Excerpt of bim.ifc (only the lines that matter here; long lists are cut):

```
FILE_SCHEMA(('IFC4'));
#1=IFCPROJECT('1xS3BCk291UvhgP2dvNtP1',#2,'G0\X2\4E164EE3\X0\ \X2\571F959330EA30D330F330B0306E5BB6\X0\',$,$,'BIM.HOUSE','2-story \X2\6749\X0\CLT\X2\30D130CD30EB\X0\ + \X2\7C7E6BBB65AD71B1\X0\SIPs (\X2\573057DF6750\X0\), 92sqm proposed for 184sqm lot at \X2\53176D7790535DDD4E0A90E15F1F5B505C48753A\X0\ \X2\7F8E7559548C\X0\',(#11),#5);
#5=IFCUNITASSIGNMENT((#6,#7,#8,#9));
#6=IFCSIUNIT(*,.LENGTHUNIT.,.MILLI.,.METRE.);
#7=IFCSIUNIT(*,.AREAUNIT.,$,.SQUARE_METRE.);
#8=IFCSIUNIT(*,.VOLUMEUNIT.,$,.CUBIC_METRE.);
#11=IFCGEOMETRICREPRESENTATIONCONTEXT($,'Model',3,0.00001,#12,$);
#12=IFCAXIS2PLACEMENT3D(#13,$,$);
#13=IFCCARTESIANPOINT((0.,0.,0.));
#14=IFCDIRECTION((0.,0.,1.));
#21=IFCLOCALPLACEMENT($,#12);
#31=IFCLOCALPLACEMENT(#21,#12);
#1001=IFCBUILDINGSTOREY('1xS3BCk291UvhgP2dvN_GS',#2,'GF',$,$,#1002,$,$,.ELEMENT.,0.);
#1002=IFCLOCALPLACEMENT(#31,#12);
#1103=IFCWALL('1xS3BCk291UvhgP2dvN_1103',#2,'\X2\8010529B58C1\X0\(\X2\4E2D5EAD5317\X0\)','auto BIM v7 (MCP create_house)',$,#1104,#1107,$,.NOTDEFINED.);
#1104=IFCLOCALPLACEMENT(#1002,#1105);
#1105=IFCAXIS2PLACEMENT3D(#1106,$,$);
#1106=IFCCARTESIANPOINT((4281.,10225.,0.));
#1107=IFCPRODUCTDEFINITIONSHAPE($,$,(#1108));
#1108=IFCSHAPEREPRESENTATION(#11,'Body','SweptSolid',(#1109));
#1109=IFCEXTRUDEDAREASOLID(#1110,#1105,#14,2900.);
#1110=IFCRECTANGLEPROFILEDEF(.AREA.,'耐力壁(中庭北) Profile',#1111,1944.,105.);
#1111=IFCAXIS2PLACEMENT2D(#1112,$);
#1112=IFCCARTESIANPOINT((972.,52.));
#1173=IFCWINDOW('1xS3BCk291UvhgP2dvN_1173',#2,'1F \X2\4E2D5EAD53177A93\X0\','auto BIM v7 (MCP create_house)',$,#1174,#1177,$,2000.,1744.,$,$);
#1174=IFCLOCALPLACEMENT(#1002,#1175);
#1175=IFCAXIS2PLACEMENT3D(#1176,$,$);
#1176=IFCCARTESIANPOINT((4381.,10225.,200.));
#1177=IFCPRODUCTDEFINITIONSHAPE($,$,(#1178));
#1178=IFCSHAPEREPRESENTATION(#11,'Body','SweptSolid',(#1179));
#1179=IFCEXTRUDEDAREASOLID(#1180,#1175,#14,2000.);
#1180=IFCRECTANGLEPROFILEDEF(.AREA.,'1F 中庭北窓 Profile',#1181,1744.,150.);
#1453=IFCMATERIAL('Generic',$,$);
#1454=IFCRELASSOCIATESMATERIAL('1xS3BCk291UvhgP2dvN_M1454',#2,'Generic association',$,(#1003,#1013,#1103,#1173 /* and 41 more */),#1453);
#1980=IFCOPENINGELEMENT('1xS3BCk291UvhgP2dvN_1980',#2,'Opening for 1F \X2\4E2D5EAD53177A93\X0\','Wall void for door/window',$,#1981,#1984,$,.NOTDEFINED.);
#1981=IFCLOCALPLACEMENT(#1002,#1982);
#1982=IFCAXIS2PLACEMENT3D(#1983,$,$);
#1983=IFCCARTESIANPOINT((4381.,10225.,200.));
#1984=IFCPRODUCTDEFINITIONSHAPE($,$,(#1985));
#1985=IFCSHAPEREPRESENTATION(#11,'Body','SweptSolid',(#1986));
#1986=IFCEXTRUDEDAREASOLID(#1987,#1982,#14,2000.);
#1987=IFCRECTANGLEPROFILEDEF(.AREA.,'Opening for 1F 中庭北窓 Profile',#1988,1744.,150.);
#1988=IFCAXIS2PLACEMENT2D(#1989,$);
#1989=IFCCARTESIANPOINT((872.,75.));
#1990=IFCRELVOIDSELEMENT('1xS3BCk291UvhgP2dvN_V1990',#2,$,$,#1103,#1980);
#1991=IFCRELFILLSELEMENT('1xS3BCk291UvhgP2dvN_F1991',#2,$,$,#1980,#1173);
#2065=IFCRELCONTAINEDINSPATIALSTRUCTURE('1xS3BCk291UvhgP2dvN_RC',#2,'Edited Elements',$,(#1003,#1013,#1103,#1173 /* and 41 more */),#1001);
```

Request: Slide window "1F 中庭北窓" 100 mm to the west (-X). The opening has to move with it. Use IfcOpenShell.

```python
import ifcopenshell
import ifcopenshell.api.geometry
import ifcopenshell.util.placement
import ifcopenshell.util.unit

model = ifcopenshell.open("bim.ifc")
unit_scale = ifcopenshell.util.unit.calculate_unit_scale(model)

window = model.by_guid("1xS3BCk291UvhgP2dvN_1173")
opening = window.FillsVoids[0].RelatingOpeningElement
wall = opening.VoidsElements[0].RelatingBuildingElement

wall_matrix = ifcopenshell.util.placement.get_local_placement(wall.ObjectPlacement)
shift = wall_matrix[:3, 0] * -0.1 / unit_scale
before = ifcopenshell.util.placement.get_local_placement(window.ObjectPlacement)[:3, 3].copy()

# The window is not placed relative to its opening, so move both.
for product in (opening, window):
    matrix = ifcopenshell.util.placement.get_local_placement(product.ObjectPlacement)
    matrix[:3, 3] += shift
    ifcopenshell.api.geometry.edit_object_placement(model, product=product, matrix=matrix, is_si=False)

after = ifcopenshell.util.placement.get_local_placement(window.ObjectPlacement)[:3, 3]
print("window moved by", (after - before).round(3) + 0.0)

model.write("bim_updated.ifc")
```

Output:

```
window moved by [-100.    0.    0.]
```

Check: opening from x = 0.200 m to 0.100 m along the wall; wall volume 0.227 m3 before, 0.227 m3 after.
